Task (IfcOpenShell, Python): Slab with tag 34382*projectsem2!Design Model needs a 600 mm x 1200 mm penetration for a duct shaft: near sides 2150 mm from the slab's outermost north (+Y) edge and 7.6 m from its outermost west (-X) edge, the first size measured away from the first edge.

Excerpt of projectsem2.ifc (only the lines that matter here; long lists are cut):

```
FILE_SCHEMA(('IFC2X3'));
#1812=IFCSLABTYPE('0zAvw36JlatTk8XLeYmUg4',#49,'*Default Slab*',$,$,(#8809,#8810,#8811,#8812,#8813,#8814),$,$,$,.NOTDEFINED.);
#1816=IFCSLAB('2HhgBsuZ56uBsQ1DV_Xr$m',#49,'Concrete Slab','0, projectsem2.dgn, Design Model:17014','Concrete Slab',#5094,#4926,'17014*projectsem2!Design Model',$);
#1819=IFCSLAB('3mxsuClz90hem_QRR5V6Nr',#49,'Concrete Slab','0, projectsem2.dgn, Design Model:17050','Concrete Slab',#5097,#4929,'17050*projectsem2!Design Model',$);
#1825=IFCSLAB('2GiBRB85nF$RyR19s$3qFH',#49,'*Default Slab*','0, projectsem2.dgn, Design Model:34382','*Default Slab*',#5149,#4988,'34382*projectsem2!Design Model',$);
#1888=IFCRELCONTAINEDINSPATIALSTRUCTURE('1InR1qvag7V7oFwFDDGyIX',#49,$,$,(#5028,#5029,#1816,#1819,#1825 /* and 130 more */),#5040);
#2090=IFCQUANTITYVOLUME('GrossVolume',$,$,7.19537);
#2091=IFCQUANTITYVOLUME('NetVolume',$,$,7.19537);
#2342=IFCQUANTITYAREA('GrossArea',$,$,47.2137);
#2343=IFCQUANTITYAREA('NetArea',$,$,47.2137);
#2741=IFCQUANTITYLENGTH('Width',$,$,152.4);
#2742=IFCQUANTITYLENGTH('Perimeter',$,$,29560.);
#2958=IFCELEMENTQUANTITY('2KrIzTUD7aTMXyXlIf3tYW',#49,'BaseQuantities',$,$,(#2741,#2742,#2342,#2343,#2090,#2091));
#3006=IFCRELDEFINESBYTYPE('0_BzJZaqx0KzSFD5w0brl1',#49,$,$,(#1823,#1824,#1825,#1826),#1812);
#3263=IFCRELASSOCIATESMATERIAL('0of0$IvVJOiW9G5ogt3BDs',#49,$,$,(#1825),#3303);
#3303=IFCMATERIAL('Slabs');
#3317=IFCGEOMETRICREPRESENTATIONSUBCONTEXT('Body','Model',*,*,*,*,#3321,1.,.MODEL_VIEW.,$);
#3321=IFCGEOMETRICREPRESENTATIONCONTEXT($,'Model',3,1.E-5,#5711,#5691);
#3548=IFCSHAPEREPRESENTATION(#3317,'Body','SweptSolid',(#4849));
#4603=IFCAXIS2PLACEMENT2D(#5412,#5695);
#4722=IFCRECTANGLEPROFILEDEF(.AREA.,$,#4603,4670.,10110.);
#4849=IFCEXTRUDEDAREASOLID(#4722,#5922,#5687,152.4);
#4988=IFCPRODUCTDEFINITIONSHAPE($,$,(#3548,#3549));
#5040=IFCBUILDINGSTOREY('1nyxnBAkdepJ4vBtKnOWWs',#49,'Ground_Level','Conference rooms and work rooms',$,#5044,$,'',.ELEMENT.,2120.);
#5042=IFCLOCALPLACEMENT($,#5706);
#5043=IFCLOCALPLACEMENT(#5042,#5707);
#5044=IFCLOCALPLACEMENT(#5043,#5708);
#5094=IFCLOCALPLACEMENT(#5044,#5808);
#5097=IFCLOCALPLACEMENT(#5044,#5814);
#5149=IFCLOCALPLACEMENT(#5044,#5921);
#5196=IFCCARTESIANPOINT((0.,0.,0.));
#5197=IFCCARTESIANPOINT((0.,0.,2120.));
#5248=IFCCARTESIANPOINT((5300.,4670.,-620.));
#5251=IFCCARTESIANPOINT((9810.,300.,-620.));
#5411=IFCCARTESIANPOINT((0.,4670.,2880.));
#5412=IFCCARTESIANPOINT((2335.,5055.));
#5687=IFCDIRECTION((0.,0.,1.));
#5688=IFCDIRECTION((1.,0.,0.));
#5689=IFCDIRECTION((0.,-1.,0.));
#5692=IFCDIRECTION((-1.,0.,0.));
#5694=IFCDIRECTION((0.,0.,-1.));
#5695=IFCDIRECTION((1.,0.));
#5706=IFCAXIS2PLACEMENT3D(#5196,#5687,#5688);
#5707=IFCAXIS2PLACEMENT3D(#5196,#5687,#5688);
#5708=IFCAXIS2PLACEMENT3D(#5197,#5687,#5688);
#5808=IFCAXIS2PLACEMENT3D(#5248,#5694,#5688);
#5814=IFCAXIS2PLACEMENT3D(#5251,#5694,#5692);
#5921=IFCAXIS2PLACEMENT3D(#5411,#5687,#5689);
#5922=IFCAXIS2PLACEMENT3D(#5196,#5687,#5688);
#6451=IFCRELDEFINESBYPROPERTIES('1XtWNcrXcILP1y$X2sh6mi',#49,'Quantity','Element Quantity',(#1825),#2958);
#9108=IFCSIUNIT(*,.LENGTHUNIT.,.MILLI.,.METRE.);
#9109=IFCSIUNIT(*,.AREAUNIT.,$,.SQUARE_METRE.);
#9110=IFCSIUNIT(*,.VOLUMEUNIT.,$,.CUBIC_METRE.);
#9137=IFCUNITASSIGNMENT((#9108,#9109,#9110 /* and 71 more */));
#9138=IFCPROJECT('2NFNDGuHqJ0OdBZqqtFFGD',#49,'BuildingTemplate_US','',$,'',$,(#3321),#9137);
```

```python
import numpy as np
import ifcopenshell
import ifcopenshell.api.feature
import ifcopenshell.api.geometry
import ifcopenshell.api.pset
import ifcopenshell.api.root
import ifcopenshell.geom
import ifcopenshell.util.element
import ifcopenshell.util.placement
import ifcopenshell.util.representation
import ifcopenshell.util.shape
import ifcopenshell.util.unit

model = ifcopenshell.open("projectsem2.ifc")
unit_scale = ifcopenshell.util.unit.calculate_unit_scale(model)
area_scale = ifcopenshell.util.unit.calculate_unit_scale(model, "AREAUNIT")
volume_scale = ifcopenshell.util.unit.calculate_unit_scale(model, "VOLUMEUNIT")
settings = ifcopenshell.geom.settings()


def volume(element):
    """Net volume in cubic metres, openings subtracted."""
    shape = ifcopenshell.geom.create_shape(settings, element)
    return ifcopenshell.util.shape.get_volume(shape.geometry)


slab = model.by_id(1825)
before = volume(slab)

# Extent in the slab's own axes, in metres. The edges named are its -X and -Y sides.
slab_shape = ifcopenshell.geom.create_shape(settings, slab)
vertices = ifcopenshell.util.shape.get_vertices(slab_shape.geometry)
x_min, y_min, bottom = vertices.min(axis=0)
top = vertices[:, 2].max()

opening = ifcopenshell.api.root.create_entity(model, ifc_class="IfcOpeningElement", name="Duct shaft opening")
context = ifcopenshell.util.representation.get_context(model, "Model", "Body", "MODEL_VIEW")
width, depth = 0.6, 1.2
outline = [(0.0, 0.0), (width, 0.0), (width, depth), (0.0, depth), (0.0, 0.0)]
# Overshoot both faces by 50 mm so the cut is clean.
shape = ifcopenshell.api.geometry.add_slab_representation(
    model, context=context, depth=top - bottom + 0.1, polyline=outline
)
ifcopenshell.api.geometry.assign_representation(model, product=opening, representation=shape)

matrix = ifcopenshell.util.placement.get_local_placement(slab.ObjectPlacement)
matrix[:, 3] = matrix @ np.append(np.array([x_min + 2.15, y_min + 7.6, bottom - 0.05]) / unit_scale, 1.0)
ifcopenshell.api.geometry.edit_object_placement(model, product=opening, matrix=matrix, is_si=False)
ifcopenshell.api.feature.add_feature(model, feature=opening, element=slab)

after = volume(slab)

# Update the slab's stored quantities.
qto = model.by_id(ifcopenshell.util.element.get_pset(slab, "BaseQuantities", should_inherit=False)["id"])
ifcopenshell.api.pset.edit_qto(model, qto=qto, properties={
    "NetArea": after / (top - bottom) / area_scale,
    "NetVolume": after / volume_scale,
})

print(f"slab volume {before:.3f} -> {after:.3f} m3")

model.write("projectsem2-out.ifc")
```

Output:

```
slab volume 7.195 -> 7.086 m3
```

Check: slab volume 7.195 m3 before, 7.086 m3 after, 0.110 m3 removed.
